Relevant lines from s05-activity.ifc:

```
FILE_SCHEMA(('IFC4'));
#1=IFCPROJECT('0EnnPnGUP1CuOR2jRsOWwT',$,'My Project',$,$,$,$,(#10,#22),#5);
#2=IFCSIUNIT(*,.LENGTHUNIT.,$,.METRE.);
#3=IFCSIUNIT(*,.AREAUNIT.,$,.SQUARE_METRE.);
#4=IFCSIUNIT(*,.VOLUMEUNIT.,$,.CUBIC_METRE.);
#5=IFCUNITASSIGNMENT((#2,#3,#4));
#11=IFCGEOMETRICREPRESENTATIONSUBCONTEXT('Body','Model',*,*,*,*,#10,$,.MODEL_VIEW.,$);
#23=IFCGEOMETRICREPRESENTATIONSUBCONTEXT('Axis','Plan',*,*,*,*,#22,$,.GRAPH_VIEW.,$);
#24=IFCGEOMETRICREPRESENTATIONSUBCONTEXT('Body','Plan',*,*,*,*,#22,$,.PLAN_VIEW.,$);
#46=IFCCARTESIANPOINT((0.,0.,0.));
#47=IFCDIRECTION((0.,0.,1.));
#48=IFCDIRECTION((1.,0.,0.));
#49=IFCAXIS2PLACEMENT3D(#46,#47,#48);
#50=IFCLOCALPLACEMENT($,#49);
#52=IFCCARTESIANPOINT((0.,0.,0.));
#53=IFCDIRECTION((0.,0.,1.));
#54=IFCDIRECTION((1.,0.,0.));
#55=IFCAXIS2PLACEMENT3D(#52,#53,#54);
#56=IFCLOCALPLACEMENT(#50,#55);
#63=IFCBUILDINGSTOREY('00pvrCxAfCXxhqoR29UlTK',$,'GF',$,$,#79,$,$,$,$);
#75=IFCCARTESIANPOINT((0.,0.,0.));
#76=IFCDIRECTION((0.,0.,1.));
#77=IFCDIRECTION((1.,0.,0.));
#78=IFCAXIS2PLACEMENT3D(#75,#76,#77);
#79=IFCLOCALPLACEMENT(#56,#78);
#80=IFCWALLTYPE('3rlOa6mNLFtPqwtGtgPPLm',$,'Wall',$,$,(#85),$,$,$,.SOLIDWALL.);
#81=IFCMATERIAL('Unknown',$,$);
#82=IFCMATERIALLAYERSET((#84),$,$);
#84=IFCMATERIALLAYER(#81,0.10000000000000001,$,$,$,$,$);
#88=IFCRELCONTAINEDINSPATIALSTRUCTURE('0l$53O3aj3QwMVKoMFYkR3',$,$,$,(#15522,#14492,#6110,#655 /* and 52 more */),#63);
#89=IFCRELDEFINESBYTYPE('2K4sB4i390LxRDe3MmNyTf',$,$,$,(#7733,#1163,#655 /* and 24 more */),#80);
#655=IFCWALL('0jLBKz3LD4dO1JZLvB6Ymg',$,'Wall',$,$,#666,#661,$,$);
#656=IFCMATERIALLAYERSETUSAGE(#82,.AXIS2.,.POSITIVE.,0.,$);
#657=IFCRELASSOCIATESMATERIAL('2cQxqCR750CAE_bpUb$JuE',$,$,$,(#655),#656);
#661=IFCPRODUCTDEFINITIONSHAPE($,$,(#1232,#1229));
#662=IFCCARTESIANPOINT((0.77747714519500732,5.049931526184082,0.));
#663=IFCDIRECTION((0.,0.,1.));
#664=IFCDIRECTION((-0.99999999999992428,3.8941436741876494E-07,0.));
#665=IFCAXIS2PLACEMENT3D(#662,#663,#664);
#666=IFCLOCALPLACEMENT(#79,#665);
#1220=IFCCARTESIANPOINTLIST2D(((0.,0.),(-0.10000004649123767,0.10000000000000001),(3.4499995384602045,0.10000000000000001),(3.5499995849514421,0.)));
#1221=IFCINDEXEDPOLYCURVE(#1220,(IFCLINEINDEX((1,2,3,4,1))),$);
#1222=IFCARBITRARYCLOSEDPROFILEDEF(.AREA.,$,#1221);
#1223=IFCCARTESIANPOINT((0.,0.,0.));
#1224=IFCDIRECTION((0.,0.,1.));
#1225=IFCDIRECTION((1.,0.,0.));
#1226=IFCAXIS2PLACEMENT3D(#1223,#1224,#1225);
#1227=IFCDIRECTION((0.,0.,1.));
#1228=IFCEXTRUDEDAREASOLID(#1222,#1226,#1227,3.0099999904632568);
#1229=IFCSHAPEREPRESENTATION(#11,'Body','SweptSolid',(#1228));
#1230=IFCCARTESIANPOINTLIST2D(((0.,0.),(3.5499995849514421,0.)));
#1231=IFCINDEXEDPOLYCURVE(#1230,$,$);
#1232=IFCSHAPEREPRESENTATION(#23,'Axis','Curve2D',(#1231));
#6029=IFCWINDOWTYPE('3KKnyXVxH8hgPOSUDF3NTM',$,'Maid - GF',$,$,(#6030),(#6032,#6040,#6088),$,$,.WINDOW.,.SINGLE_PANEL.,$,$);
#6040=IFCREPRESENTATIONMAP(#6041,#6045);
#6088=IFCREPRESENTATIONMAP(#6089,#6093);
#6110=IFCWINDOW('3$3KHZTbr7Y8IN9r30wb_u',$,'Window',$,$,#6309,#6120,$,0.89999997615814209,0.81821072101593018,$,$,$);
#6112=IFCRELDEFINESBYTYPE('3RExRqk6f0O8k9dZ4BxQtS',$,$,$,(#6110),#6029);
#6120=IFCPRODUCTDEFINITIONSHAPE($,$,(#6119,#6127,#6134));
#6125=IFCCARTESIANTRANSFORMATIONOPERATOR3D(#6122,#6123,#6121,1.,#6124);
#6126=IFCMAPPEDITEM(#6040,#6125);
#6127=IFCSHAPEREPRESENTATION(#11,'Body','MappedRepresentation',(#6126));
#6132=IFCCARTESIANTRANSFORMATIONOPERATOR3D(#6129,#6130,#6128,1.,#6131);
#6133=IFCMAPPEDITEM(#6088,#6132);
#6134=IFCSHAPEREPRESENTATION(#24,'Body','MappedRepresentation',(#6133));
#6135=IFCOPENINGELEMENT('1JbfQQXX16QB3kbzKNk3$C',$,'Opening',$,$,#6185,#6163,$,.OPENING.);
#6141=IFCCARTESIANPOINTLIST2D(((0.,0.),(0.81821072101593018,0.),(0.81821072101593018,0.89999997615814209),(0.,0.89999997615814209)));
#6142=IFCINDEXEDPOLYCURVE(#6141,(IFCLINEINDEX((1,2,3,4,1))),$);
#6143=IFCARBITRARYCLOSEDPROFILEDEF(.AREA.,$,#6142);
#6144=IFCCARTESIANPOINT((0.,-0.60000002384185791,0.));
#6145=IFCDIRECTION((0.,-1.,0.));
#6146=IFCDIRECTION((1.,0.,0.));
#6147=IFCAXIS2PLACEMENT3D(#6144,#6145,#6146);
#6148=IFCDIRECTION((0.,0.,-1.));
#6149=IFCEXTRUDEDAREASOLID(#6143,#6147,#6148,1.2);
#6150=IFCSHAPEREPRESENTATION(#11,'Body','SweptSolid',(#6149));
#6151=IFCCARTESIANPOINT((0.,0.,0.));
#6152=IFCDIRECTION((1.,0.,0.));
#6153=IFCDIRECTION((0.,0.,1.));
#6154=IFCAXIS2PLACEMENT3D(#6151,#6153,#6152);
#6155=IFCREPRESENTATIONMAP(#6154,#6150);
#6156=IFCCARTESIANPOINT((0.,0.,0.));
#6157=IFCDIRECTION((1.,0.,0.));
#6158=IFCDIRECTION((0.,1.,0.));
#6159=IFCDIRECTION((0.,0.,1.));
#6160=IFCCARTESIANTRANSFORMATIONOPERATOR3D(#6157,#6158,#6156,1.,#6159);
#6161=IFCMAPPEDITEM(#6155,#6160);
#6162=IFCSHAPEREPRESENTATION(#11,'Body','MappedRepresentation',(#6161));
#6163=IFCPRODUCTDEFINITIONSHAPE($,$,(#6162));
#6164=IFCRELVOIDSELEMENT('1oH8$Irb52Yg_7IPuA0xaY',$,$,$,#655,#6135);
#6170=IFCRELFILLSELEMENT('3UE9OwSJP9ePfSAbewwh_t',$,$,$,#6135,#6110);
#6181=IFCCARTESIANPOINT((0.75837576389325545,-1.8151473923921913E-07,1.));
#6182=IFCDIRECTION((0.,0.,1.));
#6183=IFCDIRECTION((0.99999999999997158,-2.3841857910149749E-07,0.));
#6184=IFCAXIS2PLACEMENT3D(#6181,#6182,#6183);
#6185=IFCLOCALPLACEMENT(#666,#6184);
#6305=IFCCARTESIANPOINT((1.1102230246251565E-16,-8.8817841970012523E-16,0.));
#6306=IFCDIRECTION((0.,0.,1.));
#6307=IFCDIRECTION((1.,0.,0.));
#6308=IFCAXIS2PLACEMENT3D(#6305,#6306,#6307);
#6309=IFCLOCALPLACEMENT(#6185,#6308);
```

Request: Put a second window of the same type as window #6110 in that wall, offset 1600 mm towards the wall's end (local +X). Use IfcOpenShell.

```python
import ifcopenshell
import ifcopenshell.api.feature
import ifcopenshell.api.geometry
import ifcopenshell.api.root
import ifcopenshell.geom
import ifcopenshell.util.element
import ifcopenshell.util.placement
import ifcopenshell.util.shape
import ifcopenshell.util.unit

model = ifcopenshell.open("s05-activity.ifc")
unit_scale = ifcopenshell.util.unit.calculate_unit_scale(model)
settings = ifcopenshell.geom.settings()


def volume(element):
    """Net volume in cubic metres, openings subtracted."""
    shape = ifcopenshell.geom.create_shape(settings, element)
    return ifcopenshell.util.shape.get_volume(shape.geometry)


window = model.by_guid("3$3KHZTbr7Y8IN9r30wb_u")
opening = window.FillsVoids[0].RelatingOpeningElement
wall = opening.VoidsElements[0].RelatingBuildingElement
before = volume(wall)
shift = ifcopenshell.util.placement.get_local_placement(wall.ObjectPlacement)[:3, 0] * 1.6 / unit_scale

# copy_class copies the void relationship, type, container and properties, but no geometry.
new_opening = ifcopenshell.api.root.copy_class(model, product=opening)
new_opening.Representation = ifcopenshell.util.element.copy_deep(
    model, opening.Representation, exclude=["IfcGeometricRepresentationContext", "IfcRepresentationMap"]
)
new_window = ifcopenshell.api.root.copy_class(model, product=window)
new_window.Representation = ifcopenshell.util.element.copy_deep(
    model, window.Representation, exclude=["IfcGeometricRepresentationContext", "IfcRepresentationMap"]
)
ifcopenshell.api.feature.add_filling(model, opening=new_opening, element=new_window)

for old, new in ((opening, new_opening), (window, new_window)):
    matrix = ifcopenshell.util.placement.get_local_placement(old.ObjectPlacement)
    matrix[:3, 3] += shift
    ifcopenshell.api.geometry.edit_object_placement(model, product=new, matrix=matrix, is_si=False)

after = volume(wall)

print(f"wall volume {before:.3f} -> {after:.3f} m3")

model.write("s05-activity_edited.ifc")
```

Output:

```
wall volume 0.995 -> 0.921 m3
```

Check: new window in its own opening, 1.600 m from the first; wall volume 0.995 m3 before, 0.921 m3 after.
